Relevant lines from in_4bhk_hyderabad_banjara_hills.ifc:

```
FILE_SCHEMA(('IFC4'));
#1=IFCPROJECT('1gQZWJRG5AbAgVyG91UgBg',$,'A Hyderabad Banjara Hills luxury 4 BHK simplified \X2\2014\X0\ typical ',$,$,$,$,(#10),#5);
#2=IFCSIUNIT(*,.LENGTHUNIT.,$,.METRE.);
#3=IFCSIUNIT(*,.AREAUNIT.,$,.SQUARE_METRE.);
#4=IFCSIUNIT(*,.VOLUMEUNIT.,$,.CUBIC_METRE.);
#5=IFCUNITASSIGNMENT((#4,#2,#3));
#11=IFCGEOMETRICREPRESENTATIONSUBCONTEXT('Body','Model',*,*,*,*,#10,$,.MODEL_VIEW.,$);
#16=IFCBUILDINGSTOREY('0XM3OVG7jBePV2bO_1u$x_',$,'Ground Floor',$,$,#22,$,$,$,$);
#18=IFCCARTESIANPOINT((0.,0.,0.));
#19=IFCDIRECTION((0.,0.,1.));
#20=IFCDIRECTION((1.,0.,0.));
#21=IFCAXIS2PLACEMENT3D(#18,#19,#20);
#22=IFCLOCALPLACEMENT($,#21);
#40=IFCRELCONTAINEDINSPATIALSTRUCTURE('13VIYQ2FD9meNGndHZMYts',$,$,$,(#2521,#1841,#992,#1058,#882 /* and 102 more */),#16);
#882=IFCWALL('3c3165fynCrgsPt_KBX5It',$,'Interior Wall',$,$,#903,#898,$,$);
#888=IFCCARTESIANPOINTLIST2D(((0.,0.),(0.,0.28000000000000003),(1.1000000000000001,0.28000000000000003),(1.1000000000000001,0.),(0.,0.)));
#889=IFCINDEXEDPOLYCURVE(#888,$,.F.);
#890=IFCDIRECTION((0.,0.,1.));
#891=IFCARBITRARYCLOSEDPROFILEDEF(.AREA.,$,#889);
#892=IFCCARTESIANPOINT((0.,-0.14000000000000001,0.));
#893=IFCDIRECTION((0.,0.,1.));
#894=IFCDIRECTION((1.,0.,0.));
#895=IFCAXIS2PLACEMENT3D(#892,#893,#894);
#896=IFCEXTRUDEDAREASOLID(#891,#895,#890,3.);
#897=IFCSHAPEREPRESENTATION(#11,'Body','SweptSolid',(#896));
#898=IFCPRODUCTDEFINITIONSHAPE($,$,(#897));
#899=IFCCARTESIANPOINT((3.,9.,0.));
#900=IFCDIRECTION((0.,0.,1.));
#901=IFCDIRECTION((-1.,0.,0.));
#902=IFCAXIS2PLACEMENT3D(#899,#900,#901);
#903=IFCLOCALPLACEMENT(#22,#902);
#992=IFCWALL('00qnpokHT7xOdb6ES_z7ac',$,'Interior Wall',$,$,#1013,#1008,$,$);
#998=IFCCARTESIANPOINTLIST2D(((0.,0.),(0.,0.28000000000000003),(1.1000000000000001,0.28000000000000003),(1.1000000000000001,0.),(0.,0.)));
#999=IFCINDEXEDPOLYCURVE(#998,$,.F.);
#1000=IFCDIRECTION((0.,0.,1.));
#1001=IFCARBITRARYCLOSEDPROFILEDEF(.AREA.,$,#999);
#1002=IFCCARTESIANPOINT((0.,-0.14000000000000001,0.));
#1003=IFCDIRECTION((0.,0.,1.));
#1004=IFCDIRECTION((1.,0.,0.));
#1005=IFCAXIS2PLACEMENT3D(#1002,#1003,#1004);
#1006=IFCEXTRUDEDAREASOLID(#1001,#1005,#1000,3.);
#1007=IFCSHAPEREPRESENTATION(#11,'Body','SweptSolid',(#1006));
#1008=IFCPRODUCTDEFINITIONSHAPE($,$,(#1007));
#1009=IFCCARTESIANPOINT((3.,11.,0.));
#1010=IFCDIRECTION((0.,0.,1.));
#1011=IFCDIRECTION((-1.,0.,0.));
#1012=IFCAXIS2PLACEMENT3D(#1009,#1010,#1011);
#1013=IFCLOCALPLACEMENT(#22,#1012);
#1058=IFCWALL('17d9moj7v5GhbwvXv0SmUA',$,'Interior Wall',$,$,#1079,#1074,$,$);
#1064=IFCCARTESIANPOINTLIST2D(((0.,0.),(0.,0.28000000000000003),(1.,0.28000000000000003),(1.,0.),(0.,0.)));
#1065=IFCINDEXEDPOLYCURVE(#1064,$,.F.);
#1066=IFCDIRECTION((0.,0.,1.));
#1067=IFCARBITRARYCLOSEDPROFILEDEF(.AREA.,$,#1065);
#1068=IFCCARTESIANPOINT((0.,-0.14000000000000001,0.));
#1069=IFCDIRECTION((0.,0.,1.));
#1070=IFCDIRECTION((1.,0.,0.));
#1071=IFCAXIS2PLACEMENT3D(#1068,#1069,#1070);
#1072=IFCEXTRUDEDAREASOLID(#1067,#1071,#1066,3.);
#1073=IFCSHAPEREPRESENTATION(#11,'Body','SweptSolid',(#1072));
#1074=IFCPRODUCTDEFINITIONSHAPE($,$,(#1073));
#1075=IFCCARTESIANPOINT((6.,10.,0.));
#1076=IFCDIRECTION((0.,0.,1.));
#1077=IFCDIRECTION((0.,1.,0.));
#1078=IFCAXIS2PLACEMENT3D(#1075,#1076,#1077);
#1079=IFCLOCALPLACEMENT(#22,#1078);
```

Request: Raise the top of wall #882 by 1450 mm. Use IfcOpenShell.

```python
import ifcopenshell
import ifcopenshell.geom
import ifcopenshell.util.representation
import ifcopenshell.util.shape
import ifcopenshell.util.unit

model = ifcopenshell.open("in_4bhk_hyderabad_banjara_hills.ifc")
unit_scale = ifcopenshell.util.unit.calculate_unit_scale(model)
settings = ifcopenshell.geom.settings()


def volume(element):
    """Net volume in cubic metres, openings subtracted."""
    shape = ifcopenshell.geom.create_shape(settings, element)
    return ifcopenshell.util.shape.get_volume(shape.geometry)


wall = model.by_guid("3c3165fynCrgsPt_KBX5It")
before = volume(wall)

body = ifcopenshell.util.representation.get_representation(wall, "Model", "Body")
solid = body.Items[0]
old_height = solid.Depth
solid.Depth += 1.45 / unit_scale
after = volume(wall)

print(f"height {old_height:g} -> {solid.Depth:g}, volume {before:.3f} -> {after:.3f} m3")

model.write("in_4bhk_hyderabad_banjara_hills_v2.ifc")
```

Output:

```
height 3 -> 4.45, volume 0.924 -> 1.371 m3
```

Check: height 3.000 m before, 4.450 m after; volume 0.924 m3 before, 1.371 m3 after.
